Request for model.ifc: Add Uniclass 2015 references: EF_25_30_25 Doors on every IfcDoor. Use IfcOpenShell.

First a look at what the model holds.

```python
import ifcopenshell

model = ifcopenshell.open("model.ifc")
print(model.schema)
print("classifications:", [c.Name for c in model.by_type("IfcClassification")])
for ifc_class in ("IfcDoor", "IfcRoof", "IfcStair", "IfcWall", "IfcWindow"):
    print(ifc_class, len(model.by_type(ifc_class)))
```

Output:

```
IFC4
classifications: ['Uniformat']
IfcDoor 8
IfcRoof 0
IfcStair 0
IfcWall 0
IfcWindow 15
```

```python
import ifcopenshell
import ifcopenshell.api.classification

model = ifcopenshell.open("model.ifc")

system = ifcopenshell.api.classification.add_classification(model, classification="Uniclass 2015")

codes = {
    "IfcDoor": ("EF_25_30_25", "Doors"),
}
for ifc_class, (code, name) in codes.items():
    products = model.by_type(ifc_class)
    ifcopenshell.api.classification.add_reference(
        model, products=products, classification=system, identification=code, name=name
    )
    print(code, len(products))

model.write("model_rev.ifc")
```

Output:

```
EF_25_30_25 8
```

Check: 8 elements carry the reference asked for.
